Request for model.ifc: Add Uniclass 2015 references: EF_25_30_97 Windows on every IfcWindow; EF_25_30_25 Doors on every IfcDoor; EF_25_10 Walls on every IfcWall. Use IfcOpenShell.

First a look at what the model holds.

```python
import ifcopenshell

model = ifcopenshell.open("model.ifc")
print(model.schema)
print("classifications:", [c.Name for c in model.by_type("IfcClassification")])
for ifc_class in ("IfcDoor", "IfcRoof", "IfcStair", "IfcWall", "IfcWindow"):
    print(ifc_class, len(model.by_type(ifc_class)))
```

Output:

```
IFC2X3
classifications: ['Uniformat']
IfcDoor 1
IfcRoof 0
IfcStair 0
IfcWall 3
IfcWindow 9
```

```python
import ifcopenshell
import ifcopenshell.api.classification

model = ifcopenshell.open("model.ifc")

# IFC2X3 requires Source and Edition and has no link from the project to the system.
system = model.create_entity("IfcClassification", Source="NBS", Edition="2015", Name="Uniclass 2015")

codes = {
    "IfcWindow": ("EF_25_30_97", "Windows"),
    "IfcDoor": ("EF_25_30_25", "Doors"),
    "IfcWall": ("EF_25_10", "Walls"),
}
for ifc_class, (code, name) in codes.items():
    products = model.by_type(ifc_class)
    ifcopenshell.api.classification.add_reference(
        model, products=products, classification=system, identification=code, name=name
    )
    print(code, len(products))

model.write("model_rev.ifc")
```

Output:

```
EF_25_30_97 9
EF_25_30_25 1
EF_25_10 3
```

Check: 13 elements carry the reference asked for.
